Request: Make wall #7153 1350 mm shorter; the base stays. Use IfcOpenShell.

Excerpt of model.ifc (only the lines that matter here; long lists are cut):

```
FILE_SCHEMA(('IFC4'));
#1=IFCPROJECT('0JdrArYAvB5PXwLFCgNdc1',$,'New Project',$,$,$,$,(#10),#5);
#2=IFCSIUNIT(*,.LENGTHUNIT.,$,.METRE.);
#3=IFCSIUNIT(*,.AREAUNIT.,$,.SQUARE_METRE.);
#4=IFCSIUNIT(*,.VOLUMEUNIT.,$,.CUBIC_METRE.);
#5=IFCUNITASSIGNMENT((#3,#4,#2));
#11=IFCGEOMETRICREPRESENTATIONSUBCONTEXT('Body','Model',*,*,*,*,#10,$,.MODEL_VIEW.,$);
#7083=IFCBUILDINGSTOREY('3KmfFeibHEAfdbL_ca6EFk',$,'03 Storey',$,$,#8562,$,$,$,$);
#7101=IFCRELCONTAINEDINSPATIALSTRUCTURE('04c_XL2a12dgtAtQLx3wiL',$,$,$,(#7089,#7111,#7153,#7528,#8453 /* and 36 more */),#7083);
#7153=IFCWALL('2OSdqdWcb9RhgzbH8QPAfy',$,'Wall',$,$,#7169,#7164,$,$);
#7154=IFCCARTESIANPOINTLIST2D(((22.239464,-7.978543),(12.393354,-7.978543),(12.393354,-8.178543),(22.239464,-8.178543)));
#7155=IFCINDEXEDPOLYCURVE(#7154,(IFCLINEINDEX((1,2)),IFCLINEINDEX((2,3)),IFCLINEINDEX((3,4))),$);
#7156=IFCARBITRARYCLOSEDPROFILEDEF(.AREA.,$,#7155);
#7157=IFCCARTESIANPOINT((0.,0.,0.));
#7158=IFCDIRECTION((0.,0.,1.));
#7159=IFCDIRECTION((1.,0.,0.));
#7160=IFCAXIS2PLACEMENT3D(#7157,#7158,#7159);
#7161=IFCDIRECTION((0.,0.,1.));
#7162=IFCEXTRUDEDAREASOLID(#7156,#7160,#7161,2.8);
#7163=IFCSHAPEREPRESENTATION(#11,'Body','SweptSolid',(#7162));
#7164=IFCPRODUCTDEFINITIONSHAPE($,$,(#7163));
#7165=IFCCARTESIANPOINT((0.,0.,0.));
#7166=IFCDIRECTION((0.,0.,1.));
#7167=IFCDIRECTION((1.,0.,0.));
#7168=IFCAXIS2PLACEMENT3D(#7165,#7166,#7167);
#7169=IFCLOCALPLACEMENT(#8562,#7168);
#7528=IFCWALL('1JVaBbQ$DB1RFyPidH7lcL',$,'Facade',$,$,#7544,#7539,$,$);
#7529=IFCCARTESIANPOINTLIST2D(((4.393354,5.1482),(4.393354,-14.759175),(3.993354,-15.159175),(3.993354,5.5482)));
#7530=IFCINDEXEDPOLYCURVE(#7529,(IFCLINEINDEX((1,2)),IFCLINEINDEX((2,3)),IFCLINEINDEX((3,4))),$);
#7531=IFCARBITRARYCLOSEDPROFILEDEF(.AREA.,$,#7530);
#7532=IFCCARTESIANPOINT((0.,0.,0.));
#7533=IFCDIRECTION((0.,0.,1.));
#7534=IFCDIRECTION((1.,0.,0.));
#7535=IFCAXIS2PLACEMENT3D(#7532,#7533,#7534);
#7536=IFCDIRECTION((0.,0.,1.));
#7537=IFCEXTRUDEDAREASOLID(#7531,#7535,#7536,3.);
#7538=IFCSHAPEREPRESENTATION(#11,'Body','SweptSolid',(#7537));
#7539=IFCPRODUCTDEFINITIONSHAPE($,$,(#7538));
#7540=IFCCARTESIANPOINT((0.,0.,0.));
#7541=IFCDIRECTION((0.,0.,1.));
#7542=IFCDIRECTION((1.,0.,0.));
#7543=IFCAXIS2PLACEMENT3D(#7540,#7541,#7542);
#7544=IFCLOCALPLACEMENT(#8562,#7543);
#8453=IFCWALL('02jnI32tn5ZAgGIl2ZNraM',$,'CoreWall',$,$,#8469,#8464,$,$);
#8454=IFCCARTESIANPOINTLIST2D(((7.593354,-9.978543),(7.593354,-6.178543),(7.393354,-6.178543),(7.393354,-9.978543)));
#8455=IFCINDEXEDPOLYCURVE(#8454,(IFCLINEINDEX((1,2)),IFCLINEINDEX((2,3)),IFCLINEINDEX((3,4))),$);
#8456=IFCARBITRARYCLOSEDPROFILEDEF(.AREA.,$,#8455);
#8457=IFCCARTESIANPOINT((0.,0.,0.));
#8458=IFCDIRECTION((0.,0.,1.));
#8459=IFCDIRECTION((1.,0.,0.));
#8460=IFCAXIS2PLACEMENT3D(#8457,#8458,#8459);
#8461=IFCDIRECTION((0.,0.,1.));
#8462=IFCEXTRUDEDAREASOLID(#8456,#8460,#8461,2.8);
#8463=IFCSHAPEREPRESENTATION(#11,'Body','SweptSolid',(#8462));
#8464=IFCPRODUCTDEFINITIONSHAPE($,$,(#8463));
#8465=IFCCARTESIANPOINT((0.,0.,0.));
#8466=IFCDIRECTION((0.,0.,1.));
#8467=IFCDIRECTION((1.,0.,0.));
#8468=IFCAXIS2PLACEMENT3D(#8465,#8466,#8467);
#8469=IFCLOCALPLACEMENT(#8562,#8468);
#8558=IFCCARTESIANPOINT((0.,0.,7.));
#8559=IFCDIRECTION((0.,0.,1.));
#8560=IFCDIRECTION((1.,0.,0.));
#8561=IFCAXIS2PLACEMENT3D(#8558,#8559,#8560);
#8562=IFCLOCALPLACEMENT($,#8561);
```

```python
import ifcopenshell
import ifcopenshell.geom
import ifcopenshell.util.representation
import ifcopenshell.util.shape
import ifcopenshell.util.unit

model = ifcopenshell.open("model.ifc")
unit_scale = ifcopenshell.util.unit.calculate_unit_scale(model)
settings = ifcopenshell.geom.settings()


def volume(element):
    """Net volume in cubic metres, openings subtracted."""
    shape = ifcopenshell.geom.create_shape(settings, element)
    return ifcopenshell.util.shape.get_volume(shape.geometry)


wall = model.by_guid("2OSdqdWcb9RhgzbH8QPAfy")
before = volume(wall)

body = ifcopenshell.util.representation.get_representation(wall, "Model", "Body")
solid = body.Items[0]
old_height = solid.Depth
solid.Depth -= 1.35 / unit_scale
after = volume(wall)

print(f"height {old_height:g} -> {solid.Depth:g}, volume {before:.3f} -> {after:.3f} m3")

model.write("model_edited.ifc")
```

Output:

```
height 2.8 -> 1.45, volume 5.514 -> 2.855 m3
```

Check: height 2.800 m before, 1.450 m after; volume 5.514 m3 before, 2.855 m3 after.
